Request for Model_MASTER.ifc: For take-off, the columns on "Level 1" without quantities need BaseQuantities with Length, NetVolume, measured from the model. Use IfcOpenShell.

First a look at what the model holds.

```python
import ifcopenshell
import ifcopenshell.util.element
import ifcopenshell.util.unit

model = ifcopenshell.open("Model_MASTER.ifc")
print(model.schema)
for unit_type in ("LENGTHUNIT", "AREAUNIT", "VOLUMEUNIT"):
    print(unit_type, ifcopenshell.util.unit.calculate_unit_scale(model, unit_type))
storey = next(s for s in model.by_type("IfcBuildingStorey") if s.Name == "Level 1")
columns = [e for e in ifcopenshell.util.element.get_decomposition(storey) if e.is_a("IfcColumn")]
for e in sorted(columns, key=lambda e: e.id()):
    print(e.id(), e.is_a(), e.Name, list(ifcopenshell.util.element.get_psets(e, qtos_only=True)), sep=" | ")
```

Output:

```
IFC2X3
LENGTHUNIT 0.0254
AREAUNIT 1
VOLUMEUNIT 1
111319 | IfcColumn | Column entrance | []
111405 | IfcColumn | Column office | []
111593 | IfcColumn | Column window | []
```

```python
import ifcopenshell
import ifcopenshell.api.pset
import ifcopenshell.geom
import ifcopenshell.util.element
import ifcopenshell.util.shape
import ifcopenshell.util.unit

model = ifcopenshell.open("Model_MASTER.ifc")
unit_scale = ifcopenshell.util.unit.calculate_unit_scale(model)
volume_scale = ifcopenshell.util.unit.calculate_unit_scale(model, "VOLUMEUNIT")
settings = ifcopenshell.geom.settings()

storey = next(s for s in model.by_type("IfcBuildingStorey") if s.Name == "Level 1")
columns = [e for e in ifcopenshell.util.element.get_decomposition(storey) if e.is_a("IfcColumn")]

for e in sorted(columns, key=lambda e: e.id()):
    if ifcopenshell.util.element.get_psets(e, qtos_only=True, should_inherit=False):
        continue
    # Geometry comes back in metres, in the element's own axes.
    shape = ifcopenshell.geom.create_shape(settings, e)
    values = {
        "Length": ifcopenshell.util.shape.get_z(shape.geometry) / unit_scale,
        "NetVolume": ifcopenshell.util.shape.get_volume(shape.geometry) / volume_scale,
    }
    qto = ifcopenshell.api.pset.add_qto(model, product=e, name="BaseQuantities")
    ifcopenshell.api.pset.edit_qto(model, qto=qto, properties=values)
    print(e.id(), {k: round(v, 3) for k, v in values.items()})

model.write("Model_MASTER_edited.ifc")
```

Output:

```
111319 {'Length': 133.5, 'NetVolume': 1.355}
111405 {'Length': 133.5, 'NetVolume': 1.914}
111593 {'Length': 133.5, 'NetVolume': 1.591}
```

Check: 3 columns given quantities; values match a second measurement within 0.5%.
